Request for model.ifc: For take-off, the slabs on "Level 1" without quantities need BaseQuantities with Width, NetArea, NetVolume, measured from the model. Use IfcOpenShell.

First a look at what the model holds.

```python
import ifcopenshell
import ifcopenshell.util.element
import ifcopenshell.util.unit

model = ifcopenshell.open("model.ifc")
print(model.schema)
for unit_type in ("LENGTHUNIT", "AREAUNIT", "VOLUMEUNIT"):
    print(unit_type, ifcopenshell.util.unit.calculate_unit_scale(model, unit_type))
storey = next(s for s in model.by_type("IfcBuildingStorey") if s.Name == "Level 1")
slabs = [e for e in ifcopenshell.util.element.get_decomposition(storey) if e.is_a("IfcSlab")]
for e in sorted(slabs, key=lambda e: e.id()):
    print(e.id(), e.is_a(), e.Name, list(ifcopenshell.util.element.get_psets(e, qtos_only=True)), sep=" | ")
```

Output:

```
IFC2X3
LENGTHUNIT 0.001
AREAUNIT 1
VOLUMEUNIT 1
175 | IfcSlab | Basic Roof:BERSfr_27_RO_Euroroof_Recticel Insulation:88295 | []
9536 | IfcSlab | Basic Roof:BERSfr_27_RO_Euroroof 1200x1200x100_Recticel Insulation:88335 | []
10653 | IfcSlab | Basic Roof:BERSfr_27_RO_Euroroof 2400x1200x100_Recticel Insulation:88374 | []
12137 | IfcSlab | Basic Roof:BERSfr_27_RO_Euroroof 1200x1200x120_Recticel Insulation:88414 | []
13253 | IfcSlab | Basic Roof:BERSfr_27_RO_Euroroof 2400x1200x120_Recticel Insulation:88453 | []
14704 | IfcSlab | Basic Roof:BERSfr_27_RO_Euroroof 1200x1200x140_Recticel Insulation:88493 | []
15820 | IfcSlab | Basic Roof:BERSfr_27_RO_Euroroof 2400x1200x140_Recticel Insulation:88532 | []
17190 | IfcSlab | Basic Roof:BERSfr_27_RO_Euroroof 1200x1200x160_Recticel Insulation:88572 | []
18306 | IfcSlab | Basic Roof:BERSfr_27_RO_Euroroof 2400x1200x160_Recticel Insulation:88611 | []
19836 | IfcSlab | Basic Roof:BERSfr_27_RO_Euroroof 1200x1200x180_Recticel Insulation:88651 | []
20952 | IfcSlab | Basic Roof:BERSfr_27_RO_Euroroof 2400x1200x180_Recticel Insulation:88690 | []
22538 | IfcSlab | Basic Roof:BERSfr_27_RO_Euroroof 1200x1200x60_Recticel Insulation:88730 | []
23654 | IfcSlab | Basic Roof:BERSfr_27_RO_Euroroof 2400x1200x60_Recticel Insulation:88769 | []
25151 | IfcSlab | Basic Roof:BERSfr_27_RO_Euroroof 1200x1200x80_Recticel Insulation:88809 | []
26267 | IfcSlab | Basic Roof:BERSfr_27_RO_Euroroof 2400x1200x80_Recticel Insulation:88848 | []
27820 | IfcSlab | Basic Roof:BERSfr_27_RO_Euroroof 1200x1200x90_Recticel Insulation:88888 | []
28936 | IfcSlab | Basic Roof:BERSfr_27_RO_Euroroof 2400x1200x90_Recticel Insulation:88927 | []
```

```python
import ifcopenshell
import ifcopenshell.api.pset
import ifcopenshell.geom
import ifcopenshell.util.element
import ifcopenshell.util.shape
import ifcopenshell.util.unit

model = ifcopenshell.open("model.ifc")
unit_scale = ifcopenshell.util.unit.calculate_unit_scale(model)
area_scale = ifcopenshell.util.unit.calculate_unit_scale(model, "AREAUNIT")
volume_scale = ifcopenshell.util.unit.calculate_unit_scale(model, "VOLUMEUNIT")
settings = ifcopenshell.geom.settings()

storey = next(s for s in model.by_type("IfcBuildingStorey") if s.Name == "Level 1")
slabs = [e for e in ifcopenshell.util.element.get_decomposition(storey) if e.is_a("IfcSlab")]

for e in sorted(slabs, key=lambda e: e.id()):
    if ifcopenshell.util.element.get_psets(e, qtos_only=True, should_inherit=False):
        continue
    # Geometry comes back in metres, in the element's own axes.
    shape = ifcopenshell.geom.create_shape(settings, e)
    values = {
        "Width": ifcopenshell.util.shape.get_z(shape.geometry) / unit_scale,
        "NetArea": ifcopenshell.util.shape.get_footprint_area(shape.geometry) / area_scale,
        "NetVolume": ifcopenshell.util.shape.get_volume(shape.geometry) / volume_scale,
    }
    qto = ifcopenshell.api.pset.add_qto(model, product=e, name="BaseQuantities")
    ifcopenshell.api.pset.edit_qto(model, qto=qto, properties=values)
    print(e.id(), {k: round(v, 3) for k, v in values.items()})

model.write("model_v2.ifc")
```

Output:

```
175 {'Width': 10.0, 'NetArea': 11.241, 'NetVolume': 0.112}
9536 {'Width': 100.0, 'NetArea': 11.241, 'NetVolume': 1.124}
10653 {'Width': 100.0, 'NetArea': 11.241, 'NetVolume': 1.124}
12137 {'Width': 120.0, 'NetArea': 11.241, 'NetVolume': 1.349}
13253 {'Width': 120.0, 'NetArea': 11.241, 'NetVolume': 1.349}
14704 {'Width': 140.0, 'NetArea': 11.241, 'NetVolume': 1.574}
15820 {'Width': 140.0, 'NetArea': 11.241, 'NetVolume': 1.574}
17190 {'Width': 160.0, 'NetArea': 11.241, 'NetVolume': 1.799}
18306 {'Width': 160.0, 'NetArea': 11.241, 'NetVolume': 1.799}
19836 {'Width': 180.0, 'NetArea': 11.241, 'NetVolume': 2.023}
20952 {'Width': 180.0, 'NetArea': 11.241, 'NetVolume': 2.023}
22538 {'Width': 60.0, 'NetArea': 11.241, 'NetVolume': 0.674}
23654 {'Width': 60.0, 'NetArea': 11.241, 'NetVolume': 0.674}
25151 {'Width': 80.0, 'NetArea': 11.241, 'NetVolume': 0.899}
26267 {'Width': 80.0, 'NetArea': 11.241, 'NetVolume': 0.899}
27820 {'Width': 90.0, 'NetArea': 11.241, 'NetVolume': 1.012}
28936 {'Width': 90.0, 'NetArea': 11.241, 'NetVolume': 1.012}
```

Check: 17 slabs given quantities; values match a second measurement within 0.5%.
